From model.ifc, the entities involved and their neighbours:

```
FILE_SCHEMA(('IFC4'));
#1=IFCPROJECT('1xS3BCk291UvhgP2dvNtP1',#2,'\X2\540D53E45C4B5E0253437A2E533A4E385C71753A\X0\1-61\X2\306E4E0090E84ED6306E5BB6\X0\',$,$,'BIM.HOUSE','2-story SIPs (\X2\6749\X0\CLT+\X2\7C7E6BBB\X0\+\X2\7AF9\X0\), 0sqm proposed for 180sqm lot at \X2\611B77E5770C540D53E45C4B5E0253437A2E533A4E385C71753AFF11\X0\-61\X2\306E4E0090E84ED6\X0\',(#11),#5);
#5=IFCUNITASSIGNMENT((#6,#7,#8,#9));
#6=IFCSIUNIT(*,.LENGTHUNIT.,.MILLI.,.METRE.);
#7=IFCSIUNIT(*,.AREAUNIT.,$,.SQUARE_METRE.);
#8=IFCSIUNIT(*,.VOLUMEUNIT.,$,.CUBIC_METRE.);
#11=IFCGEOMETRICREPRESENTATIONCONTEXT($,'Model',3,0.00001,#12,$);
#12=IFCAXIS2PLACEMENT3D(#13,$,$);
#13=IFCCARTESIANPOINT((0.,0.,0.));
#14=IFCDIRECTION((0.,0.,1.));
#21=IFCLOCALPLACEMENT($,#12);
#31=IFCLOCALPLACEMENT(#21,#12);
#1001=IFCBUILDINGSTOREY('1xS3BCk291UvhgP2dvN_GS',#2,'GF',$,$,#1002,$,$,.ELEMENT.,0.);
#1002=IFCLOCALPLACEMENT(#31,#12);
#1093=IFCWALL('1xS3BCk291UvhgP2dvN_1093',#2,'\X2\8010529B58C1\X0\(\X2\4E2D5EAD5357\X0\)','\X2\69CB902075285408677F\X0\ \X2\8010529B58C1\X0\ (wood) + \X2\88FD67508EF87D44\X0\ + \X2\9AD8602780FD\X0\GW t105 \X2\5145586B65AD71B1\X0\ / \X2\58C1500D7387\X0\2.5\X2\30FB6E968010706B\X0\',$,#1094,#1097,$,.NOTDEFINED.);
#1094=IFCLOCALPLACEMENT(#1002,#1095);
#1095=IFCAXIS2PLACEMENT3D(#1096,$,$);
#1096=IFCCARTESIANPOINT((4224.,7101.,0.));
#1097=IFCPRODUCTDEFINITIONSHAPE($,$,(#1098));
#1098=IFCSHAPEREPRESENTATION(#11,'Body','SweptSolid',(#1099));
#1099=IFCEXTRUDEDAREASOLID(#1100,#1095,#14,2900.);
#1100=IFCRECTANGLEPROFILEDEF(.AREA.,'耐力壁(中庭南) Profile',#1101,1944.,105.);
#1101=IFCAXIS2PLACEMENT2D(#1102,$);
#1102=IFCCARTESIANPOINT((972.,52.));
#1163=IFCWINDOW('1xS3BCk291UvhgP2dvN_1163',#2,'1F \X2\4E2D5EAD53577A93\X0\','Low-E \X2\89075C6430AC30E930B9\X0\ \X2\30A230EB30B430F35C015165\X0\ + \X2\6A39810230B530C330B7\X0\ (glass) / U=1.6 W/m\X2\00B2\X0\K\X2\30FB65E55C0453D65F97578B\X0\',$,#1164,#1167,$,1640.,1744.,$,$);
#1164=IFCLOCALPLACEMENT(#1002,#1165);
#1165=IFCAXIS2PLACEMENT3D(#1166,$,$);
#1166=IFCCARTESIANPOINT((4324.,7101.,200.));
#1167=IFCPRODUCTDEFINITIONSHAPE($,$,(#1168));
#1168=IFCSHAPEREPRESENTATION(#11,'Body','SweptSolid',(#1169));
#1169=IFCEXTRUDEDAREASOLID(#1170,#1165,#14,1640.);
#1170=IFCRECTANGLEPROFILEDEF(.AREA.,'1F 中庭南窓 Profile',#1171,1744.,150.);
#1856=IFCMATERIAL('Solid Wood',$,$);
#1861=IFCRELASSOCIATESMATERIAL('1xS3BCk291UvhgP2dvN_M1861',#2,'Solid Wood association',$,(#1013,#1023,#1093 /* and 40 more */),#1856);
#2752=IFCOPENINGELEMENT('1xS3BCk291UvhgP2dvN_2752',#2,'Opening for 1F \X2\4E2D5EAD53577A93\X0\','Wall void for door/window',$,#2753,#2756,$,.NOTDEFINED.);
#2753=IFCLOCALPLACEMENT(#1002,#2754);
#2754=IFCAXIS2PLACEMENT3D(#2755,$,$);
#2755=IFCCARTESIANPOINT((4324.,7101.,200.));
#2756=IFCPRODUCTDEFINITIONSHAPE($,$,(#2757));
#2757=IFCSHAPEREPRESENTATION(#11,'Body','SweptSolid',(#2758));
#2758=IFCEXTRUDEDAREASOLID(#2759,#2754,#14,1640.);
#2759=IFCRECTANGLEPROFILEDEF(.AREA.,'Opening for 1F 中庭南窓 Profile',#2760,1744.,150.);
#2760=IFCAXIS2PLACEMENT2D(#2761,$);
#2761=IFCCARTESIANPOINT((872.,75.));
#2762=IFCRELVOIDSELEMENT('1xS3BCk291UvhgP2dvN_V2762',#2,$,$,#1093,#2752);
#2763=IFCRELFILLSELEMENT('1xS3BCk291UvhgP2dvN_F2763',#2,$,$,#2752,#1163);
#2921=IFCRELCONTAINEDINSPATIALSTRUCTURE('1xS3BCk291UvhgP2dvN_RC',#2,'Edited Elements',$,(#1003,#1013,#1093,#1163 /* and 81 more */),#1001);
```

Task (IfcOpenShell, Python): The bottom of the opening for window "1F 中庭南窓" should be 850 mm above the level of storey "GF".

```python
import numpy as np
import ifcopenshell
import ifcopenshell.api.geometry
import ifcopenshell.geom
import ifcopenshell.util.element
import ifcopenshell.util.placement
import ifcopenshell.util.shape
import ifcopenshell.util.unit

model = ifcopenshell.open("model.ifc")
unit_scale = ifcopenshell.util.unit.calculate_unit_scale(model)

window = model.by_guid("1xS3BCk291UvhgP2dvN_1163")
opening = window.FillsVoids[0].RelatingOpeningElement
storey = ifcopenshell.util.element.get_container(window, ifc_class="IfcBuildingStorey")
level = ifcopenshell.util.placement.get_local_placement(storey.ObjectPlacement)[2, 3]

# The opening's origin need not be at the sill, so measure its lowest point.
shape = ifcopenshell.geom.create_shape(ifcopenshell.geom.settings(), opening)
bottom = ifcopenshell.util.shape.get_shape_bottom_elevation(shape, shape.geometry) / unit_scale
dz = level + 850.0 - bottom

shift = np.array([0.0, 0.0, dz])
# The window is not placed relative to its opening, so move both.
for product in (opening, window):
    matrix = ifcopenshell.util.placement.get_local_placement(product.ObjectPlacement)
    matrix[:3, 3] += shift
    ifcopenshell.api.geometry.edit_object_placement(model, product=product, matrix=matrix, is_si=False)

print(f"moved by {dz * unit_scale:+.3f} m")

model.write("model-out.ifc")
```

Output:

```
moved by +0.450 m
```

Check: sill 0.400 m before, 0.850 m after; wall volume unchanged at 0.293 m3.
